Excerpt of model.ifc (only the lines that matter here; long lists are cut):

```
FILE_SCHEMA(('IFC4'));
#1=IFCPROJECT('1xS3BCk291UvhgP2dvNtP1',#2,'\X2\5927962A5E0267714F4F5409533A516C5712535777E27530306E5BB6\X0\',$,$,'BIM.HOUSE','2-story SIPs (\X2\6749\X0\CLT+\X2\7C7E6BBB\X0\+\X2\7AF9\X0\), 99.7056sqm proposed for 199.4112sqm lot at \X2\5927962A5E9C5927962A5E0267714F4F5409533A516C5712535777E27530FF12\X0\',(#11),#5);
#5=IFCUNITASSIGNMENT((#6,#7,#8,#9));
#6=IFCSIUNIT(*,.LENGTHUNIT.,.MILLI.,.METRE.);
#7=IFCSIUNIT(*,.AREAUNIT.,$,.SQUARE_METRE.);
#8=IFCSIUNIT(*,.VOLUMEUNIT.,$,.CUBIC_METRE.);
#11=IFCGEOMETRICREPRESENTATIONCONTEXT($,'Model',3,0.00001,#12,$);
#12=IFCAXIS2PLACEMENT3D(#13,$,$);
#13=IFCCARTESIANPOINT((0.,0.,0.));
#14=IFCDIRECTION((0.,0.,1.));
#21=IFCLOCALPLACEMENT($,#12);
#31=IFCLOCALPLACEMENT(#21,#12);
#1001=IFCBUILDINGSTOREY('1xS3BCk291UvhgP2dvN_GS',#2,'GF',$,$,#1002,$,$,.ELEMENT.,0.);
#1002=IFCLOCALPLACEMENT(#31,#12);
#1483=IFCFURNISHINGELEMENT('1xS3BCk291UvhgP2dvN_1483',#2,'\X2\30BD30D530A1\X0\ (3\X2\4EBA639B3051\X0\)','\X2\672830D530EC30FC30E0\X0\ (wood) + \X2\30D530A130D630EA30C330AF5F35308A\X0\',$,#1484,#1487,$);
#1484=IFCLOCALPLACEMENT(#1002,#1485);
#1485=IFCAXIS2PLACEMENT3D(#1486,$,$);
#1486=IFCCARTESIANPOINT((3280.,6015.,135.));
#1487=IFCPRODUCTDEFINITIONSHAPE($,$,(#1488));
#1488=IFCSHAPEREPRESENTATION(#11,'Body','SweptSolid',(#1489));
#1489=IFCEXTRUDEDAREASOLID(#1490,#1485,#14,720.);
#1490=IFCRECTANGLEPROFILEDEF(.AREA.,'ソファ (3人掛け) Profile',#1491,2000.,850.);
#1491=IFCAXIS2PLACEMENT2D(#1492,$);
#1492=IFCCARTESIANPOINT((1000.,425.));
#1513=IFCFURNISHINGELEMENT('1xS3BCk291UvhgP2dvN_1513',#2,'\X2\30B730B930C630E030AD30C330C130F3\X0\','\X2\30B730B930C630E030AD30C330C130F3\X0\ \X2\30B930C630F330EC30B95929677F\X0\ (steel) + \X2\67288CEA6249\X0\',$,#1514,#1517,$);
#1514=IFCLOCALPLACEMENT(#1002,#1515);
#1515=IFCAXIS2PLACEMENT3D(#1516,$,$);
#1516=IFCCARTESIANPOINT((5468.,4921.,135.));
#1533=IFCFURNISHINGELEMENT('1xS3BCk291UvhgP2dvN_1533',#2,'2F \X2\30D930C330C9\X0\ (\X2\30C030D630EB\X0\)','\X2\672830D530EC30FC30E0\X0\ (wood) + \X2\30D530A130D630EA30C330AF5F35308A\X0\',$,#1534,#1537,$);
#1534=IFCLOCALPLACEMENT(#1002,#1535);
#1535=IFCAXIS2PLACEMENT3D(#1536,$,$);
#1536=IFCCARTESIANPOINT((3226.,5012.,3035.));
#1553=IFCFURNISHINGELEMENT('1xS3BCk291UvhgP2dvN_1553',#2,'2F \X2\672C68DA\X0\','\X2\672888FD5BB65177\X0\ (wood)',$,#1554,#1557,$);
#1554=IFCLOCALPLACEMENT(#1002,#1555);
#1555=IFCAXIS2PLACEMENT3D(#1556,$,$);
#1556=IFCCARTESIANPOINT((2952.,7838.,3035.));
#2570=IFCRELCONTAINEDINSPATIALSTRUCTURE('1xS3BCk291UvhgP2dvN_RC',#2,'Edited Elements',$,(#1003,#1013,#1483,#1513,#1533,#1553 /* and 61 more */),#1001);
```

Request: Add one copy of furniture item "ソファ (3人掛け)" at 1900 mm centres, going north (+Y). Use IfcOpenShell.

```python
import numpy as np
import ifcopenshell
import ifcopenshell.api.geometry
import ifcopenshell.api.root
import ifcopenshell.util.element
import ifcopenshell.util.placement

model = ifcopenshell.open("model.ifc")


def reuse_history(source, copy):
    """copy_class also copies each property set's owner history, people and application; keep the originals."""
    for rel in copy.IsDefinedBy:
        if rel.is_a("IfcRelDefinesByProperties") and (history := rel.RelatingPropertyDefinition.OwnerHistory):
            rel.RelatingPropertyDefinition.OwnerHistory = source.OwnerHistory
            ifcopenshell.util.element.remove_deep2(model, history)


source = model.by_guid("1xS3BCk291UvhgP2dvN_1483")
base = ifcopenshell.util.placement.get_local_placement(source.ObjectPlacement)
step = np.array([0.0, 1.0, 0.0]) * 1900.0

for i in range(1, 2):
    copy = ifcopenshell.api.root.copy_class(model, product=source)
    copy.Representation = ifcopenshell.util.element.copy_deep(
        model, source.Representation, exclude=["IfcGeometricRepresentationContext", "IfcRepresentationMap"]
    )
    reuse_history(source, copy)
    matrix = base.copy()
    matrix[:3, 3] += i * step
    print("added at", matrix[:3, 3].round(3) + 0.0)
    ifcopenshell.api.geometry.edit_object_placement(model, product=copy, matrix=matrix, is_si=False)

model.write("model_v2.ifc")
```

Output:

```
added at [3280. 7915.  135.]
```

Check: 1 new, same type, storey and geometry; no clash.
